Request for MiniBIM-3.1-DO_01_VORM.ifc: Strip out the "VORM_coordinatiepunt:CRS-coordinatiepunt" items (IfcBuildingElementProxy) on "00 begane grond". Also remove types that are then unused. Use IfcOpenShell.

First a look at what the model holds.

```python
import ifcopenshell
import ifcopenshell.util.element

model = ifcopenshell.open("MiniBIM-3.1-DO_01_VORM.ifc")
print(model.schema)
storey = next(s for s in model.by_type("IfcBuildingStorey") if s.Name == "00 begane grond")
proxies = [e for e in ifcopenshell.util.element.get_decomposition(storey) if e.is_a("IfcBuildingElementProxy")]
seen = {}
for e in proxies:
    element_type = ifcopenshell.util.element.get_type(e)
    name = element_type.Name if element_type not in (None, e) else None
    seen[name] = seen.get(name, 0) + 1
for name, count in sorted(seen.items(), key=str):
    print(count, "x", name)
```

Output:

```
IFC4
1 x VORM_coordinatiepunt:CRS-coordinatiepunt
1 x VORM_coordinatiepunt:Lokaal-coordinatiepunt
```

```python
import ifcopenshell
import ifcopenshell.api.root
import ifcopenshell.util.element

model = ifcopenshell.open("MiniBIM-3.1-DO_01_VORM.ifc")

storey = next(s for s in model.by_type("IfcBuildingStorey") if s.Name == "00 begane grond")
proxies = [e for e in ifcopenshell.util.element.get_decomposition(storey) if e.is_a("IfcBuildingElementProxy")]
targets = [e for e in proxies if (t := ifcopenshell.util.element.get_type(e)) not in (None, e) and t.Name == "VORM_coordinatiepunt:CRS-coordinatiepunt"]
types = {ifcopenshell.util.element.get_type(e) for e in targets} - {None, *targets}

for e in targets:
    ifcopenshell.api.root.remove_product(model, product=e)
print(len(targets), "removed")

unused = [t for t in types if not ifcopenshell.util.element.get_types(t)]
for t in unused:
    ifcopenshell.api.root.remove_product(model, product=t)
print(len(unused), "unused types removed")

model.write("MiniBIM-3.1-DO_01_VORM_v2.ifc")
```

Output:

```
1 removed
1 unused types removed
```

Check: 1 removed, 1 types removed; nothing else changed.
